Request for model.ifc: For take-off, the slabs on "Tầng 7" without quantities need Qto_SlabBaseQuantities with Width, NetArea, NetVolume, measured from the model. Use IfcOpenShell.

First a look at what the model holds.

```python
import ifcopenshell
import ifcopenshell.util.element
import ifcopenshell.util.unit

model = ifcopenshell.open("model.ifc")
print(model.schema)
for unit_type in ("LENGTHUNIT", "AREAUNIT", "VOLUMEUNIT"):
    print(unit_type, ifcopenshell.util.unit.calculate_unit_scale(model, unit_type))
storey = next(s for s in model.by_type("IfcBuildingStorey") if s.Name == "Tầng 7")
slabs = [e for e in ifcopenshell.util.element.get_decomposition(storey) if e.is_a("IfcSlab")]
for e in sorted(slabs, key=lambda e: e.id()):
    print(e.id(), e.is_a(), e.Name, list(ifcopenshell.util.element.get_psets(e, qtos_only=True)), sep=" | ")
```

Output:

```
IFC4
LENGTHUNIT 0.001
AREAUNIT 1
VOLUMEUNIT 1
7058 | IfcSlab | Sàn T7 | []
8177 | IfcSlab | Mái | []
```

```python
import ifcopenshell
import ifcopenshell.api.pset
import ifcopenshell.geom
import ifcopenshell.util.element
import ifcopenshell.util.shape
import ifcopenshell.util.unit

model = ifcopenshell.open("model.ifc")
unit_scale = ifcopenshell.util.unit.calculate_unit_scale(model)
area_scale = ifcopenshell.util.unit.calculate_unit_scale(model, "AREAUNIT")
volume_scale = ifcopenshell.util.unit.calculate_unit_scale(model, "VOLUMEUNIT")
settings = ifcopenshell.geom.settings()

storey = next(s for s in model.by_type("IfcBuildingStorey") if s.Name == "Tầng 7")
slabs = [e for e in ifcopenshell.util.element.get_decomposition(storey) if e.is_a("IfcSlab")]

for e in sorted(slabs, key=lambda e: e.id()):
    if ifcopenshell.util.element.get_psets(e, qtos_only=True, should_inherit=False):
        continue
    # Geometry comes back in metres, in the element's own axes.
    shape = ifcopenshell.geom.create_shape(settings, e)
    values = {
        "Width": ifcopenshell.util.shape.get_z(shape.geometry) / unit_scale,
        "NetArea": ifcopenshell.util.shape.get_footprint_area(shape.geometry) / area_scale,
        "NetVolume": ifcopenshell.util.shape.get_volume(shape.geometry) / volume_scale,
    }
    qto = ifcopenshell.api.pset.add_qto(model, product=e, name="Qto_SlabBaseQuantities")
    ifcopenshell.api.pset.edit_qto(model, qto=qto, properties=values)
    print(e.id(), {k: round(v, 3) for k, v in values.items()})

model.write("model_edited.ifc")
```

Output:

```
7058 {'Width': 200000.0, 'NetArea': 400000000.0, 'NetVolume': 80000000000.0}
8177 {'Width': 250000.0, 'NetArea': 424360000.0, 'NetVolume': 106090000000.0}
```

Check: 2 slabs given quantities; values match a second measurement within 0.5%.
